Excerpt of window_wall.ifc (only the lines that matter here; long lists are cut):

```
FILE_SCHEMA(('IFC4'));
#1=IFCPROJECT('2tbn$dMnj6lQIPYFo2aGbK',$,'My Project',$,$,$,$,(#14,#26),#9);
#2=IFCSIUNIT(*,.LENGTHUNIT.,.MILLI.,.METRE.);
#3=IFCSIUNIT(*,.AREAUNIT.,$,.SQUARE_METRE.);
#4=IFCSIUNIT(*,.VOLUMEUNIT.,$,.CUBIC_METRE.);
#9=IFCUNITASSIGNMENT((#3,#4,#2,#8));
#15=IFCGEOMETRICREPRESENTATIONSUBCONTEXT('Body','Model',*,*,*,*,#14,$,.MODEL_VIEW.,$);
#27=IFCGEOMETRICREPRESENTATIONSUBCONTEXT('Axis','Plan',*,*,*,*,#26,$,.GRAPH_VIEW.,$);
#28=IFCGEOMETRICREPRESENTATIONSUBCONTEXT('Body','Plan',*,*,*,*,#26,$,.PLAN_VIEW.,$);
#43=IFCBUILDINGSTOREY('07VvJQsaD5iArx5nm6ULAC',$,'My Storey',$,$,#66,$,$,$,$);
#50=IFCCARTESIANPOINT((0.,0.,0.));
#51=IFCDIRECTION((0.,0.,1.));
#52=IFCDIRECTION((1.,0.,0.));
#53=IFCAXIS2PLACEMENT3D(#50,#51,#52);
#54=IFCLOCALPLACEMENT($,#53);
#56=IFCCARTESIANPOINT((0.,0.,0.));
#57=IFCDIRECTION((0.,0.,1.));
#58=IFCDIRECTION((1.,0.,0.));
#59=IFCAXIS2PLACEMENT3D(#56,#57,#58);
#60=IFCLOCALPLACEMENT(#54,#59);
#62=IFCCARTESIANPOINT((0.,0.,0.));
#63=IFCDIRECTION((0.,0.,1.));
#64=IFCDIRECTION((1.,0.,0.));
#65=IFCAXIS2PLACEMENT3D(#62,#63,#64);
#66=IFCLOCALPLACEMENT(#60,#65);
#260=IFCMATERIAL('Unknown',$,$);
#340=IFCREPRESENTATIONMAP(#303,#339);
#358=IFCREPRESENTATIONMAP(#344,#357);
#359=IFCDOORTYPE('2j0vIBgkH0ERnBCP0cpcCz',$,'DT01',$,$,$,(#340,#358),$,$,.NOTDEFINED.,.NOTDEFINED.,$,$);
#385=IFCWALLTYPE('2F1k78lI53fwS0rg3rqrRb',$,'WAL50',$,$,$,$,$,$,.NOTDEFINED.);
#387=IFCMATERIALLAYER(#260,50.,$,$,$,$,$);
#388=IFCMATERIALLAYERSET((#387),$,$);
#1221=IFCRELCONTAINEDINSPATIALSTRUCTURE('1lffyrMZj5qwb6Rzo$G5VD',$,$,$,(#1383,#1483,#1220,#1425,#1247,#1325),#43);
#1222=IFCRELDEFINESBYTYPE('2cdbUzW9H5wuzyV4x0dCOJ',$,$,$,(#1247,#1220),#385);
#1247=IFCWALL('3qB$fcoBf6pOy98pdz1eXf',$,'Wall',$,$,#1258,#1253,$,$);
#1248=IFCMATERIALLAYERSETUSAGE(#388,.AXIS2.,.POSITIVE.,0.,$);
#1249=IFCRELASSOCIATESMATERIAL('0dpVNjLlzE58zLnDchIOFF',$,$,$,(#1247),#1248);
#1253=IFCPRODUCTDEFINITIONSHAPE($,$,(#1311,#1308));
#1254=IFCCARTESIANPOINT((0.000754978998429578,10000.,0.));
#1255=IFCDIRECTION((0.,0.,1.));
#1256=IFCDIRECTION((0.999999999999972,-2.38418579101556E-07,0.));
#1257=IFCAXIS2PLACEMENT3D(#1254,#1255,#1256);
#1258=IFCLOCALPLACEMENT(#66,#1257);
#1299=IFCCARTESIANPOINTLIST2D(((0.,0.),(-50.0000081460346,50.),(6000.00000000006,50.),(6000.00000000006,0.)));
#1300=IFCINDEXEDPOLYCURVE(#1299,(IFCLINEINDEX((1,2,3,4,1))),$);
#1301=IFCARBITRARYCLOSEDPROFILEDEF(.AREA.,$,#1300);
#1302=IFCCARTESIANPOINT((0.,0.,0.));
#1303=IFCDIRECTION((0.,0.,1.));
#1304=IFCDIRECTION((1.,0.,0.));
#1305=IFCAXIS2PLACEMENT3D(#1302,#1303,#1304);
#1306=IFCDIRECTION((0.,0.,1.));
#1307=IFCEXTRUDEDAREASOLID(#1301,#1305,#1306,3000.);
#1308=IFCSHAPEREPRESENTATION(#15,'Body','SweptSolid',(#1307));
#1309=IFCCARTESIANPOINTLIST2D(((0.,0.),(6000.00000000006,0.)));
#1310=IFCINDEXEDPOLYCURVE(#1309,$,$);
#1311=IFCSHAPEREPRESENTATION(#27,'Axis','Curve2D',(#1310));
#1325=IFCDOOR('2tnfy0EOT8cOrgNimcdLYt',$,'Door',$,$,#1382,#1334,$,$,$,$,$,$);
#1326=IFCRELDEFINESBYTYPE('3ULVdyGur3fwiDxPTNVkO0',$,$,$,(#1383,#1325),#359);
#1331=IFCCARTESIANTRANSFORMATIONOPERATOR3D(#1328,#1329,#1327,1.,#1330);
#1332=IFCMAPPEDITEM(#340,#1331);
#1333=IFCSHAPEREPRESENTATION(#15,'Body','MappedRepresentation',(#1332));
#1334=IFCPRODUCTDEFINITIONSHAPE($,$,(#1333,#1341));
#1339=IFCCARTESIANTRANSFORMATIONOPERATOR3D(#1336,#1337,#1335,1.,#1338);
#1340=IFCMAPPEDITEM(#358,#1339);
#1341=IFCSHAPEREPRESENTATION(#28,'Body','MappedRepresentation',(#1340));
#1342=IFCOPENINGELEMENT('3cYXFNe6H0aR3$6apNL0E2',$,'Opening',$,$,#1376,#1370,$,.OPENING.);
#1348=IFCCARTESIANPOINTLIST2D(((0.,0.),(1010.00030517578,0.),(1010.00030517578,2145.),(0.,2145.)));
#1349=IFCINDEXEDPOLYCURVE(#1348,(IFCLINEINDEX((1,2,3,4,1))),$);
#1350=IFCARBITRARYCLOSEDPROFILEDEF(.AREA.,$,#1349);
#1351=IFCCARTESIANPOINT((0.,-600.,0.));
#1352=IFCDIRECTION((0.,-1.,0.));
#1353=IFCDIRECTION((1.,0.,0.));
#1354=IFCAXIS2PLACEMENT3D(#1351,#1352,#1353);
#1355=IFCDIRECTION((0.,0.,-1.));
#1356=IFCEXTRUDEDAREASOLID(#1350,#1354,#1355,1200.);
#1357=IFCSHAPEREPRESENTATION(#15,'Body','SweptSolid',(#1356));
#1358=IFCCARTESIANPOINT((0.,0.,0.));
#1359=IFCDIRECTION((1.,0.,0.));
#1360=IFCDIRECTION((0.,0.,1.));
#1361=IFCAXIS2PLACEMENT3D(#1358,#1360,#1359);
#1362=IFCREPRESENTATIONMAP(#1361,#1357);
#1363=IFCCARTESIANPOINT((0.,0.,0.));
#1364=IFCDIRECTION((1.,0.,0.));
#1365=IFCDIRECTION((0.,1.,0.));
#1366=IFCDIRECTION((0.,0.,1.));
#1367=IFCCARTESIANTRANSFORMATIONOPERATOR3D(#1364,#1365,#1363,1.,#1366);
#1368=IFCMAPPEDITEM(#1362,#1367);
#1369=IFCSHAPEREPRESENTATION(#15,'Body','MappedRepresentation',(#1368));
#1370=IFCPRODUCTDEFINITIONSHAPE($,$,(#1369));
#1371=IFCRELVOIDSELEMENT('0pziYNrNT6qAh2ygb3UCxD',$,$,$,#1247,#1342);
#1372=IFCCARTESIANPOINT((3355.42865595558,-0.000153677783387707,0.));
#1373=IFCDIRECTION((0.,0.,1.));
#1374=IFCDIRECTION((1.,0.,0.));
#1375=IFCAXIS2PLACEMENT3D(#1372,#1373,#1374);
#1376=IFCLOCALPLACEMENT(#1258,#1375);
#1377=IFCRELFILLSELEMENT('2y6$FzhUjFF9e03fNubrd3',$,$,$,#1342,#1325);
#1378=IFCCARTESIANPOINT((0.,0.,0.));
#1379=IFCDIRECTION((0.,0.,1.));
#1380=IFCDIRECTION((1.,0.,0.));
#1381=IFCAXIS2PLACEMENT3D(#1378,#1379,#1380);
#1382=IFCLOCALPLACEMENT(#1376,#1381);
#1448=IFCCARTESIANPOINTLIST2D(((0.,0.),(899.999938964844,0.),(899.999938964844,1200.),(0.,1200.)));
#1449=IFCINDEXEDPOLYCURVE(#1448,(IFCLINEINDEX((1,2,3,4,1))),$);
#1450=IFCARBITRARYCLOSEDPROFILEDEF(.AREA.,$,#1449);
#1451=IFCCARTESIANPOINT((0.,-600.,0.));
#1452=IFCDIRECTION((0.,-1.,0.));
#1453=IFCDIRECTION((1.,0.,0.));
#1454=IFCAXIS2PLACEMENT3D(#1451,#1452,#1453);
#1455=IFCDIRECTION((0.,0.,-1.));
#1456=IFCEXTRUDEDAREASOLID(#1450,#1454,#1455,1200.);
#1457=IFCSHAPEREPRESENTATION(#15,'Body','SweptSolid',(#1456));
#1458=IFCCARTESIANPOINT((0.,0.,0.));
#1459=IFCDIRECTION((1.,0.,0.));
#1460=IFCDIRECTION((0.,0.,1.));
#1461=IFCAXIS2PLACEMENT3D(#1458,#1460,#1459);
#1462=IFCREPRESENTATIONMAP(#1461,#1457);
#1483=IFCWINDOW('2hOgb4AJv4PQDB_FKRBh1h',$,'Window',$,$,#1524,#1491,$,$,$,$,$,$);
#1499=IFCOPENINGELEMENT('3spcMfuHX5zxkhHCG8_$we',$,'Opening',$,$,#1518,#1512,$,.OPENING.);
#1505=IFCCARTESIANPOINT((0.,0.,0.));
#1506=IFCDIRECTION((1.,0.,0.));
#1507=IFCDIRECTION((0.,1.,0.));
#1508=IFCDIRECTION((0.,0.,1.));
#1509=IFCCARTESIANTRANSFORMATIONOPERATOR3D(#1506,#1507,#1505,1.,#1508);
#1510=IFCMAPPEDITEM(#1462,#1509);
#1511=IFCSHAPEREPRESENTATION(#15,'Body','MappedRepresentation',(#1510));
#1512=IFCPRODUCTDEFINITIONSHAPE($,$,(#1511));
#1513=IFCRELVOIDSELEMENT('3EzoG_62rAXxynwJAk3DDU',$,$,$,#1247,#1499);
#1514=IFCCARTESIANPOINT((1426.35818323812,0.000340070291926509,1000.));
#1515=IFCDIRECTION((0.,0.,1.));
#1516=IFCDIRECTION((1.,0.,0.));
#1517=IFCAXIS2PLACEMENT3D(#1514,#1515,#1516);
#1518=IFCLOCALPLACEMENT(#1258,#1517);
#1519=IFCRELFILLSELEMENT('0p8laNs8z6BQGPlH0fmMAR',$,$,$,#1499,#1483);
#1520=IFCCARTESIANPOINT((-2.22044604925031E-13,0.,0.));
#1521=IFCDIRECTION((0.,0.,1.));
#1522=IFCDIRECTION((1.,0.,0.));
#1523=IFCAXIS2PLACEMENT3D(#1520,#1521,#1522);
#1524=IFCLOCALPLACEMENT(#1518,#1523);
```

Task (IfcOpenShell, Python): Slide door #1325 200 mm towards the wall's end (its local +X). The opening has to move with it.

```python
import ifcopenshell
import ifcopenshell.api.geometry
import ifcopenshell.util.placement

model = ifcopenshell.open("window_wall.ifc")

door = model.by_id(1325)
opening = door.FillsVoids[0].RelatingOpeningElement
wall = opening.VoidsElements[0].RelatingBuildingElement

wall_matrix = ifcopenshell.util.placement.get_local_placement(wall.ObjectPlacement)
shift = wall_matrix[:3, 0] * 200.0
before = ifcopenshell.util.placement.get_local_placement(door.ObjectPlacement)[:3, 3].copy()

# The door is placed relative to its opening, so it follows when the opening moves.
matrix = ifcopenshell.util.placement.get_local_placement(opening.ObjectPlacement)
matrix[:3, 3] += shift
ifcopenshell.api.geometry.edit_object_placement(
    model, product=opening, matrix=matrix, is_si=False, should_transform_children=True
)

after = ifcopenshell.util.placement.get_local_placement(door.ObjectPlacement)[:3, 3]
print("door moved by", (after - before).round(3) + 0.0)

model.write("window_wall-out.ifc")
```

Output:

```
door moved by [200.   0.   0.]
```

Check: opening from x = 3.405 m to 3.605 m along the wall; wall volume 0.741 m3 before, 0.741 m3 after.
